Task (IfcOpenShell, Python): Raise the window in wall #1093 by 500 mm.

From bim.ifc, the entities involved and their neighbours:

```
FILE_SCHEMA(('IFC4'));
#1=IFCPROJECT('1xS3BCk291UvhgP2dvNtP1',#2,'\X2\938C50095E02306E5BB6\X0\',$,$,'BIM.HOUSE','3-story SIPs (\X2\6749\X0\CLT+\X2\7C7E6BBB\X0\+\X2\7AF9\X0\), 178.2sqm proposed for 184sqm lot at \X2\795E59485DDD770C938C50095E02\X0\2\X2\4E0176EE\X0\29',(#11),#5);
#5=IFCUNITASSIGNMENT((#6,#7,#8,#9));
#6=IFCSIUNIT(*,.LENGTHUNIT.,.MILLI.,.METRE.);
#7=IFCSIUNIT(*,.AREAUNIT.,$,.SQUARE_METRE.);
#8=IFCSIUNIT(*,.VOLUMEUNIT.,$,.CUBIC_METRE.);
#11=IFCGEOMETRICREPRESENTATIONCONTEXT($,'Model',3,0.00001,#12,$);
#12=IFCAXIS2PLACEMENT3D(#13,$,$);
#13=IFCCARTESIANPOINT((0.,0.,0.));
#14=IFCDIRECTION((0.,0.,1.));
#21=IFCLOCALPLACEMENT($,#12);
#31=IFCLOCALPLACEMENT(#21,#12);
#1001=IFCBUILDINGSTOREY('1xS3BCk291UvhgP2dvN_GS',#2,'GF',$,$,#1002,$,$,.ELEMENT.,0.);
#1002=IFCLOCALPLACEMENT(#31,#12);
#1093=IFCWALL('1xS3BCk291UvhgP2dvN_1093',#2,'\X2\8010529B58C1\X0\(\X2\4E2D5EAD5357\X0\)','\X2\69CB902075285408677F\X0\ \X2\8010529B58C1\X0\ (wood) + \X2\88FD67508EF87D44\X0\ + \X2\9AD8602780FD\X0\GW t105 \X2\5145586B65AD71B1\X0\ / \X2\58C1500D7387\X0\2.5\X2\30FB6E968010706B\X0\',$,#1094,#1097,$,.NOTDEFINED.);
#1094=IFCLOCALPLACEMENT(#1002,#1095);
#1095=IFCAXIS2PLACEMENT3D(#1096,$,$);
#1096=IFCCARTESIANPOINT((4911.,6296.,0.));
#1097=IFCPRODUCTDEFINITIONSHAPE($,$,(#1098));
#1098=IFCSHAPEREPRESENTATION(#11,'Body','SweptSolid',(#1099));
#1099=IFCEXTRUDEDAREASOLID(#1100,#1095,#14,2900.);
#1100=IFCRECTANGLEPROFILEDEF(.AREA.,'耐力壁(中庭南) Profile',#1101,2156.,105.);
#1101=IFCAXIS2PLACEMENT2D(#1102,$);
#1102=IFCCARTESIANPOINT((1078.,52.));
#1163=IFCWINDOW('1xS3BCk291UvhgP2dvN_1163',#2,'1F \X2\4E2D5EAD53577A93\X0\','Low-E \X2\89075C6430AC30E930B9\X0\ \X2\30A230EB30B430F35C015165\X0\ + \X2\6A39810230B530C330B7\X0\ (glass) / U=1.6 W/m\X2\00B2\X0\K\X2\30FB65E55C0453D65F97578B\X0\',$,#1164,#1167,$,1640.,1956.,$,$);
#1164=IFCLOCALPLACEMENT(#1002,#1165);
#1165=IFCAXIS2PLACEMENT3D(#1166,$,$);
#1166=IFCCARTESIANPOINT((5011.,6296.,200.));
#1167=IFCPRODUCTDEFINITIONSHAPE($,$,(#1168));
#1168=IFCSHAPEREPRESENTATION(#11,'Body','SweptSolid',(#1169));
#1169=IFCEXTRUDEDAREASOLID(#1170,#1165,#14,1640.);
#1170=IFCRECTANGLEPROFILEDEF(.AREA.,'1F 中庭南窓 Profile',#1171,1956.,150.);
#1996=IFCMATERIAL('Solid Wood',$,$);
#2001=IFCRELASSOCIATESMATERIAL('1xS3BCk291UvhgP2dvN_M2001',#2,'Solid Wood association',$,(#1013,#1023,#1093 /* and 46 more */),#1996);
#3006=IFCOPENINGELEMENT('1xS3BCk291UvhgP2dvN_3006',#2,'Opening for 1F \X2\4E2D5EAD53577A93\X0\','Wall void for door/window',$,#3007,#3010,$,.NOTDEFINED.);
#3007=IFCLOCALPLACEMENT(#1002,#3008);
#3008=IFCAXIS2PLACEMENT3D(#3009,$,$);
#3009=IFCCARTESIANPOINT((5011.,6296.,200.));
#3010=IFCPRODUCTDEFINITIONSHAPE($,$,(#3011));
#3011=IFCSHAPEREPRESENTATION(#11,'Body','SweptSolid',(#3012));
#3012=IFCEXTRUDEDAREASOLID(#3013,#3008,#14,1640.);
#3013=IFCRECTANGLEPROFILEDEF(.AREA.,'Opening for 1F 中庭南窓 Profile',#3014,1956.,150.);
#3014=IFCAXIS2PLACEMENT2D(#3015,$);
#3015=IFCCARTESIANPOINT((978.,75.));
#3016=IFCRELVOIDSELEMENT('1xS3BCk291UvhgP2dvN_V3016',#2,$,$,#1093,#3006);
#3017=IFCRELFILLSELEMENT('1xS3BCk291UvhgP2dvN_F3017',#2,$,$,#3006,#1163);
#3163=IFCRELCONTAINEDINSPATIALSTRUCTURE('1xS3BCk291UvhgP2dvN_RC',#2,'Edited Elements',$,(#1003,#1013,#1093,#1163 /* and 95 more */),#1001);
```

```python
import numpy as np
import ifcopenshell
import ifcopenshell.api.geometry
import ifcopenshell.util.placement
import ifcopenshell.util.unit

model = ifcopenshell.open("bim.ifc")
unit_scale = ifcopenshell.util.unit.calculate_unit_scale(model)

window = model.by_guid("1xS3BCk291UvhgP2dvN_1163")
opening = window.FillsVoids[0].RelatingOpeningElement
dz = 0.5 / unit_scale

shift = np.array([0.0, 0.0, dz])
# The window is not placed relative to its opening, so move both.
for product in (opening, window):
    matrix = ifcopenshell.util.placement.get_local_placement(product.ObjectPlacement)
    matrix[:3, 3] += shift
    ifcopenshell.api.geometry.edit_object_placement(model, product=product, matrix=matrix, is_si=False)

print(f"moved by {dz * unit_scale:+.3f} m")

model.write("bim_edited.ifc")
```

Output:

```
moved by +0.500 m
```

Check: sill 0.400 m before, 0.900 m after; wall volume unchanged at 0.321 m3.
